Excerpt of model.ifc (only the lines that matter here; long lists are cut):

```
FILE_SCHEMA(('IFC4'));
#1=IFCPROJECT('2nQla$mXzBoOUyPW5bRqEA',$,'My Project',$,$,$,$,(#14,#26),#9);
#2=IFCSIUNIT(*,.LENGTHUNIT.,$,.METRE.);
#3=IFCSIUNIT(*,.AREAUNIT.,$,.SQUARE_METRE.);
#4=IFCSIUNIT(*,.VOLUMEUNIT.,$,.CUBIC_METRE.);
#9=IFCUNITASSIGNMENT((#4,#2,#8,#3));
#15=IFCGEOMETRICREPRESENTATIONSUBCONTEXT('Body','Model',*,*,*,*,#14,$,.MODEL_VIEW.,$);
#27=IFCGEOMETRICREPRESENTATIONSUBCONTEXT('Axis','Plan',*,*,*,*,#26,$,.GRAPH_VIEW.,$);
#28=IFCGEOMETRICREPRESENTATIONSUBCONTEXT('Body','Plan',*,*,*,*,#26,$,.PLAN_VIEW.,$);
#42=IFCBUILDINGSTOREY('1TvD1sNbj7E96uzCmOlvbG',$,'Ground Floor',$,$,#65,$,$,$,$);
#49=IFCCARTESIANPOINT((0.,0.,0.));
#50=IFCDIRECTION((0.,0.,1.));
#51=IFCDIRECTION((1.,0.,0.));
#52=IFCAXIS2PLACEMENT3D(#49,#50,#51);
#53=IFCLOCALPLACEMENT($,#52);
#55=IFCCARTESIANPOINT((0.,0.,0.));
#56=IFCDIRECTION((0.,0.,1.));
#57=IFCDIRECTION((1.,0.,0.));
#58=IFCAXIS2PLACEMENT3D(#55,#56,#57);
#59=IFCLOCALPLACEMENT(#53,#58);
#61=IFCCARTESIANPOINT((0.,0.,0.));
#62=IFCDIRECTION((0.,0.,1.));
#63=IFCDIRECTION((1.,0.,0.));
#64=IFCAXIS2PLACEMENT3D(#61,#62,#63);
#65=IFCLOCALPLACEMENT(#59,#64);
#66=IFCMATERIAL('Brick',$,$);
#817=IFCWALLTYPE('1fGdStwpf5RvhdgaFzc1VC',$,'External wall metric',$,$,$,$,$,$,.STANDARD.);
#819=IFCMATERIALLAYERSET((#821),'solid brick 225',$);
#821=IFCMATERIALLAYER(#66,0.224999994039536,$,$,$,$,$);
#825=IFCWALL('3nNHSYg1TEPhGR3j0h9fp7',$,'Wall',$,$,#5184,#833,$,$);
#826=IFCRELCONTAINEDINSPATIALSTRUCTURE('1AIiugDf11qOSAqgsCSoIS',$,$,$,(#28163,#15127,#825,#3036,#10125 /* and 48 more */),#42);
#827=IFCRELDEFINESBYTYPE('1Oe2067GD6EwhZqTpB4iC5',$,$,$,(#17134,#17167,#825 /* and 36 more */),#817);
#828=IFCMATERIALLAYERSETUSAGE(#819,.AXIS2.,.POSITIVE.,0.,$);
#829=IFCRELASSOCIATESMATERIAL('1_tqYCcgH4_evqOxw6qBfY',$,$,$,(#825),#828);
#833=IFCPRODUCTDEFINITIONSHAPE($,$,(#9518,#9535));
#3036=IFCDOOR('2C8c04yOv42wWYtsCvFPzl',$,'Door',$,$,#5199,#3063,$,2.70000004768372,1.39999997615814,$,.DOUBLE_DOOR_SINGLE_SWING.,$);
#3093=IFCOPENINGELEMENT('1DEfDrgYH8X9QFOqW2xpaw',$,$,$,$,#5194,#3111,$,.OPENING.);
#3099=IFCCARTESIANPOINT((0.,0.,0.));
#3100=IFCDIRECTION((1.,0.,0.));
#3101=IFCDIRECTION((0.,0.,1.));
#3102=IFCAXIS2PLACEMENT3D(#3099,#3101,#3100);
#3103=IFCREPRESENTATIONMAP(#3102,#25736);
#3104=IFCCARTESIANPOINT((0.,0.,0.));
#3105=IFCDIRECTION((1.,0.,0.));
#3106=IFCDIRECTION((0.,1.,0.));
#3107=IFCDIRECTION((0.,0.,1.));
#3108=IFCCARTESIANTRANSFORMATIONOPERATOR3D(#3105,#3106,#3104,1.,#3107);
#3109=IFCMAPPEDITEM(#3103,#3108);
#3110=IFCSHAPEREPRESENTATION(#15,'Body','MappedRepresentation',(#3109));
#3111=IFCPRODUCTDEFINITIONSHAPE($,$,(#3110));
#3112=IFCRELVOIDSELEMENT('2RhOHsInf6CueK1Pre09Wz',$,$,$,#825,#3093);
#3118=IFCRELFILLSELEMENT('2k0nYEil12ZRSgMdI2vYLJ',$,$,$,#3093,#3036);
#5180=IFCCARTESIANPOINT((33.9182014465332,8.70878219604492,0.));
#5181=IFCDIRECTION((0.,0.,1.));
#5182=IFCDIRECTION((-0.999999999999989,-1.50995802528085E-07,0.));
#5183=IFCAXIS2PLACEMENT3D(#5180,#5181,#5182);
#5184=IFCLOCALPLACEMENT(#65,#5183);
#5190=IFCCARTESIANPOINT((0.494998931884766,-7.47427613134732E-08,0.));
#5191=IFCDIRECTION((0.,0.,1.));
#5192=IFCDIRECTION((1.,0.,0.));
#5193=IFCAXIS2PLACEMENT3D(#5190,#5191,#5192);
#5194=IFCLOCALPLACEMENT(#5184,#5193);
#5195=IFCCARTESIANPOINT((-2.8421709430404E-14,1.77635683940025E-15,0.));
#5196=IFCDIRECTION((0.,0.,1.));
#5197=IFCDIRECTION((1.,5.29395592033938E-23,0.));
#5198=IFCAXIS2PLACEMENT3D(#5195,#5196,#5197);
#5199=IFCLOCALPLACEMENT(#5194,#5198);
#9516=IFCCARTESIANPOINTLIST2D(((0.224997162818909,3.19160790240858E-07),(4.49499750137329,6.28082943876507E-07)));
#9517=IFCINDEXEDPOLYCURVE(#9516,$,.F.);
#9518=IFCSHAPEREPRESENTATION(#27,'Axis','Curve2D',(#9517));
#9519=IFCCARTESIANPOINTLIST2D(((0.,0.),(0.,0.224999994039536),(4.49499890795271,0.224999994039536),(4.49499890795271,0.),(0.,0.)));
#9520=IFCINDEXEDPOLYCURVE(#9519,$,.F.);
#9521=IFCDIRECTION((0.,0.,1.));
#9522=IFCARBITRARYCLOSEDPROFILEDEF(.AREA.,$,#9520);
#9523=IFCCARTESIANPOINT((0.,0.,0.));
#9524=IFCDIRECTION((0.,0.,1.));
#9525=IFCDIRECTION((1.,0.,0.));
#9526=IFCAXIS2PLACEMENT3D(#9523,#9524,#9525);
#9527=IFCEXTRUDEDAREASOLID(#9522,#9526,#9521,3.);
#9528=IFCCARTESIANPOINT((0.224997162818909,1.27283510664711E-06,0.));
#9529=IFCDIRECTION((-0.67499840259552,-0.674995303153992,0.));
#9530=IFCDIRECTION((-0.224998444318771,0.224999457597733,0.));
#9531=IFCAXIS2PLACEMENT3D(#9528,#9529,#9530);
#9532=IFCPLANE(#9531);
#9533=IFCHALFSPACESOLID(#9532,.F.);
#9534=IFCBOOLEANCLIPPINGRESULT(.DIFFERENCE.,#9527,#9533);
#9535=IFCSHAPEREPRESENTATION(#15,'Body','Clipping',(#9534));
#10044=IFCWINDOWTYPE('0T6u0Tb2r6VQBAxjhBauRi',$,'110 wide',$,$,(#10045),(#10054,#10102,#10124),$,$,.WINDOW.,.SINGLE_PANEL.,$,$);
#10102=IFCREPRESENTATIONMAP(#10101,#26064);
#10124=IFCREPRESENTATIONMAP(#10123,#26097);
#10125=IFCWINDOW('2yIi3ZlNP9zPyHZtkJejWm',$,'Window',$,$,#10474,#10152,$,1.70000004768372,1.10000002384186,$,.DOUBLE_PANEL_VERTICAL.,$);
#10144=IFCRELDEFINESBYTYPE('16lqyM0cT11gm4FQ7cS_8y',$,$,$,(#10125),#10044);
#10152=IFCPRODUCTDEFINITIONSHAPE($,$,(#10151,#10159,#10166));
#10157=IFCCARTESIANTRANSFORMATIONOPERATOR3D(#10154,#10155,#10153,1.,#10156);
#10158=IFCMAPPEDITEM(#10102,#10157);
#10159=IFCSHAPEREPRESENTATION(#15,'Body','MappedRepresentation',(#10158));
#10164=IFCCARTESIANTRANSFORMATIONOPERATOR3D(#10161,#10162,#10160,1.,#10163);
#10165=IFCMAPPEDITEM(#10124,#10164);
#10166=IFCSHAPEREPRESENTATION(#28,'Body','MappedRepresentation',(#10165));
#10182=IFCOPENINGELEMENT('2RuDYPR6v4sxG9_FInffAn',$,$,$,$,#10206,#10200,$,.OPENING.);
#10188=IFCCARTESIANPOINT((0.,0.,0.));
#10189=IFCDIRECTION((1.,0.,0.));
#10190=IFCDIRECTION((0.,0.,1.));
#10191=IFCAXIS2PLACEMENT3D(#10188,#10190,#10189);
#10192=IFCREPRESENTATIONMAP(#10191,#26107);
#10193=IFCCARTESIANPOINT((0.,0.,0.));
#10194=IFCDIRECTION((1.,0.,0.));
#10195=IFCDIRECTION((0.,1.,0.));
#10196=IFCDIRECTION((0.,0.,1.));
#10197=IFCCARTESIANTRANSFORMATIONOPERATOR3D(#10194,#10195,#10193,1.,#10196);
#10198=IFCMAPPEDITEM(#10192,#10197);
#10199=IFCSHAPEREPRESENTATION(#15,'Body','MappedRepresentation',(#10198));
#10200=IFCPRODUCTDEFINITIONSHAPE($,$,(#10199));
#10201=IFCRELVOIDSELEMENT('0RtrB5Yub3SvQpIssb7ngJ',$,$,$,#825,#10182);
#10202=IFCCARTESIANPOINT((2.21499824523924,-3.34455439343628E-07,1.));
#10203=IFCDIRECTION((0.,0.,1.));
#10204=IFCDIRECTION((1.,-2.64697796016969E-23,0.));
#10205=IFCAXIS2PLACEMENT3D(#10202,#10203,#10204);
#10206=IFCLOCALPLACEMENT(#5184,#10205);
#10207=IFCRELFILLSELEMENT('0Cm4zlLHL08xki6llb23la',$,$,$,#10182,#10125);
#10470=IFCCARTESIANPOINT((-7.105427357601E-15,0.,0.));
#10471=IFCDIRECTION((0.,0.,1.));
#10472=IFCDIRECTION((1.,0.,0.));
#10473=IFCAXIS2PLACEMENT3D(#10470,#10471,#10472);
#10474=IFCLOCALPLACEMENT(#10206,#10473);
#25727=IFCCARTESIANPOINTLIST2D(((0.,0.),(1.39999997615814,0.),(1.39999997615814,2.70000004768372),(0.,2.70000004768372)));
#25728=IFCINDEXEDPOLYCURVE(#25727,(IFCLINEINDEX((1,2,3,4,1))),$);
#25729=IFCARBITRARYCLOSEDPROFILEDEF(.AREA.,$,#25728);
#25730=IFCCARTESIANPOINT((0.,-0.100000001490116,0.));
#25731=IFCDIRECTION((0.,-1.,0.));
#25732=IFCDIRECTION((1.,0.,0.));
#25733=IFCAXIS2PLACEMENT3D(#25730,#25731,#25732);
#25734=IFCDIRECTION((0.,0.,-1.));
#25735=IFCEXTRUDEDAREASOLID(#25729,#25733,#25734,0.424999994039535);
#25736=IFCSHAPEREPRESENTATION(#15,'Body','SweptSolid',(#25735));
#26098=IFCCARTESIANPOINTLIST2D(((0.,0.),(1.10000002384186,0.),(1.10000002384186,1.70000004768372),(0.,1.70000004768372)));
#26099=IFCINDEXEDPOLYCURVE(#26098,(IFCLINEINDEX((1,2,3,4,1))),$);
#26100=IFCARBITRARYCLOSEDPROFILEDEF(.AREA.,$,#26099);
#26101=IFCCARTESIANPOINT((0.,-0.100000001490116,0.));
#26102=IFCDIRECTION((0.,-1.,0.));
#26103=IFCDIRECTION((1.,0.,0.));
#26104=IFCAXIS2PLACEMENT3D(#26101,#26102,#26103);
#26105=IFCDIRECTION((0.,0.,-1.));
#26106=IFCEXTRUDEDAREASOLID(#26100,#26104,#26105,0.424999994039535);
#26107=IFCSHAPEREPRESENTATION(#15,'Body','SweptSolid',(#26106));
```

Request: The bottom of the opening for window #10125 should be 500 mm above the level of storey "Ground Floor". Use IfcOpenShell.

```python
import numpy as np
import ifcopenshell
import ifcopenshell.api.geometry
import ifcopenshell.geom
import ifcopenshell.util.element
import ifcopenshell.util.placement
import ifcopenshell.util.shape
import ifcopenshell.util.unit

model = ifcopenshell.open("model.ifc")
unit_scale = ifcopenshell.util.unit.calculate_unit_scale(model)

window = model.by_id(10125)
opening = window.FillsVoids[0].RelatingOpeningElement
storey = ifcopenshell.util.element.get_container(window, ifc_class="IfcBuildingStorey")
level = ifcopenshell.util.placement.get_local_placement(storey.ObjectPlacement)[2, 3]

# The opening's origin need not be at the sill, so measure its lowest point.
shape = ifcopenshell.geom.create_shape(ifcopenshell.geom.settings(), opening)
bottom = ifcopenshell.util.shape.get_shape_bottom_elevation(shape, shape.geometry) / unit_scale
dz = level + 0.5 / unit_scale - bottom

shift = np.array([0.0, 0.0, dz])
# The window is placed relative to its opening, so it follows when the opening moves.
matrix = ifcopenshell.util.placement.get_local_placement(opening.ObjectPlacement)
matrix[:3, 3] += shift
ifcopenshell.api.geometry.edit_object_placement(
    model, product=opening, matrix=matrix, is_si=False, should_transform_children=True
)

print(f"moved by {dz * unit_scale:+.3f} m")

model.write("model_edited.ifc")
```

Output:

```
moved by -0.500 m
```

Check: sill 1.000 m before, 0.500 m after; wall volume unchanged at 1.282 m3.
